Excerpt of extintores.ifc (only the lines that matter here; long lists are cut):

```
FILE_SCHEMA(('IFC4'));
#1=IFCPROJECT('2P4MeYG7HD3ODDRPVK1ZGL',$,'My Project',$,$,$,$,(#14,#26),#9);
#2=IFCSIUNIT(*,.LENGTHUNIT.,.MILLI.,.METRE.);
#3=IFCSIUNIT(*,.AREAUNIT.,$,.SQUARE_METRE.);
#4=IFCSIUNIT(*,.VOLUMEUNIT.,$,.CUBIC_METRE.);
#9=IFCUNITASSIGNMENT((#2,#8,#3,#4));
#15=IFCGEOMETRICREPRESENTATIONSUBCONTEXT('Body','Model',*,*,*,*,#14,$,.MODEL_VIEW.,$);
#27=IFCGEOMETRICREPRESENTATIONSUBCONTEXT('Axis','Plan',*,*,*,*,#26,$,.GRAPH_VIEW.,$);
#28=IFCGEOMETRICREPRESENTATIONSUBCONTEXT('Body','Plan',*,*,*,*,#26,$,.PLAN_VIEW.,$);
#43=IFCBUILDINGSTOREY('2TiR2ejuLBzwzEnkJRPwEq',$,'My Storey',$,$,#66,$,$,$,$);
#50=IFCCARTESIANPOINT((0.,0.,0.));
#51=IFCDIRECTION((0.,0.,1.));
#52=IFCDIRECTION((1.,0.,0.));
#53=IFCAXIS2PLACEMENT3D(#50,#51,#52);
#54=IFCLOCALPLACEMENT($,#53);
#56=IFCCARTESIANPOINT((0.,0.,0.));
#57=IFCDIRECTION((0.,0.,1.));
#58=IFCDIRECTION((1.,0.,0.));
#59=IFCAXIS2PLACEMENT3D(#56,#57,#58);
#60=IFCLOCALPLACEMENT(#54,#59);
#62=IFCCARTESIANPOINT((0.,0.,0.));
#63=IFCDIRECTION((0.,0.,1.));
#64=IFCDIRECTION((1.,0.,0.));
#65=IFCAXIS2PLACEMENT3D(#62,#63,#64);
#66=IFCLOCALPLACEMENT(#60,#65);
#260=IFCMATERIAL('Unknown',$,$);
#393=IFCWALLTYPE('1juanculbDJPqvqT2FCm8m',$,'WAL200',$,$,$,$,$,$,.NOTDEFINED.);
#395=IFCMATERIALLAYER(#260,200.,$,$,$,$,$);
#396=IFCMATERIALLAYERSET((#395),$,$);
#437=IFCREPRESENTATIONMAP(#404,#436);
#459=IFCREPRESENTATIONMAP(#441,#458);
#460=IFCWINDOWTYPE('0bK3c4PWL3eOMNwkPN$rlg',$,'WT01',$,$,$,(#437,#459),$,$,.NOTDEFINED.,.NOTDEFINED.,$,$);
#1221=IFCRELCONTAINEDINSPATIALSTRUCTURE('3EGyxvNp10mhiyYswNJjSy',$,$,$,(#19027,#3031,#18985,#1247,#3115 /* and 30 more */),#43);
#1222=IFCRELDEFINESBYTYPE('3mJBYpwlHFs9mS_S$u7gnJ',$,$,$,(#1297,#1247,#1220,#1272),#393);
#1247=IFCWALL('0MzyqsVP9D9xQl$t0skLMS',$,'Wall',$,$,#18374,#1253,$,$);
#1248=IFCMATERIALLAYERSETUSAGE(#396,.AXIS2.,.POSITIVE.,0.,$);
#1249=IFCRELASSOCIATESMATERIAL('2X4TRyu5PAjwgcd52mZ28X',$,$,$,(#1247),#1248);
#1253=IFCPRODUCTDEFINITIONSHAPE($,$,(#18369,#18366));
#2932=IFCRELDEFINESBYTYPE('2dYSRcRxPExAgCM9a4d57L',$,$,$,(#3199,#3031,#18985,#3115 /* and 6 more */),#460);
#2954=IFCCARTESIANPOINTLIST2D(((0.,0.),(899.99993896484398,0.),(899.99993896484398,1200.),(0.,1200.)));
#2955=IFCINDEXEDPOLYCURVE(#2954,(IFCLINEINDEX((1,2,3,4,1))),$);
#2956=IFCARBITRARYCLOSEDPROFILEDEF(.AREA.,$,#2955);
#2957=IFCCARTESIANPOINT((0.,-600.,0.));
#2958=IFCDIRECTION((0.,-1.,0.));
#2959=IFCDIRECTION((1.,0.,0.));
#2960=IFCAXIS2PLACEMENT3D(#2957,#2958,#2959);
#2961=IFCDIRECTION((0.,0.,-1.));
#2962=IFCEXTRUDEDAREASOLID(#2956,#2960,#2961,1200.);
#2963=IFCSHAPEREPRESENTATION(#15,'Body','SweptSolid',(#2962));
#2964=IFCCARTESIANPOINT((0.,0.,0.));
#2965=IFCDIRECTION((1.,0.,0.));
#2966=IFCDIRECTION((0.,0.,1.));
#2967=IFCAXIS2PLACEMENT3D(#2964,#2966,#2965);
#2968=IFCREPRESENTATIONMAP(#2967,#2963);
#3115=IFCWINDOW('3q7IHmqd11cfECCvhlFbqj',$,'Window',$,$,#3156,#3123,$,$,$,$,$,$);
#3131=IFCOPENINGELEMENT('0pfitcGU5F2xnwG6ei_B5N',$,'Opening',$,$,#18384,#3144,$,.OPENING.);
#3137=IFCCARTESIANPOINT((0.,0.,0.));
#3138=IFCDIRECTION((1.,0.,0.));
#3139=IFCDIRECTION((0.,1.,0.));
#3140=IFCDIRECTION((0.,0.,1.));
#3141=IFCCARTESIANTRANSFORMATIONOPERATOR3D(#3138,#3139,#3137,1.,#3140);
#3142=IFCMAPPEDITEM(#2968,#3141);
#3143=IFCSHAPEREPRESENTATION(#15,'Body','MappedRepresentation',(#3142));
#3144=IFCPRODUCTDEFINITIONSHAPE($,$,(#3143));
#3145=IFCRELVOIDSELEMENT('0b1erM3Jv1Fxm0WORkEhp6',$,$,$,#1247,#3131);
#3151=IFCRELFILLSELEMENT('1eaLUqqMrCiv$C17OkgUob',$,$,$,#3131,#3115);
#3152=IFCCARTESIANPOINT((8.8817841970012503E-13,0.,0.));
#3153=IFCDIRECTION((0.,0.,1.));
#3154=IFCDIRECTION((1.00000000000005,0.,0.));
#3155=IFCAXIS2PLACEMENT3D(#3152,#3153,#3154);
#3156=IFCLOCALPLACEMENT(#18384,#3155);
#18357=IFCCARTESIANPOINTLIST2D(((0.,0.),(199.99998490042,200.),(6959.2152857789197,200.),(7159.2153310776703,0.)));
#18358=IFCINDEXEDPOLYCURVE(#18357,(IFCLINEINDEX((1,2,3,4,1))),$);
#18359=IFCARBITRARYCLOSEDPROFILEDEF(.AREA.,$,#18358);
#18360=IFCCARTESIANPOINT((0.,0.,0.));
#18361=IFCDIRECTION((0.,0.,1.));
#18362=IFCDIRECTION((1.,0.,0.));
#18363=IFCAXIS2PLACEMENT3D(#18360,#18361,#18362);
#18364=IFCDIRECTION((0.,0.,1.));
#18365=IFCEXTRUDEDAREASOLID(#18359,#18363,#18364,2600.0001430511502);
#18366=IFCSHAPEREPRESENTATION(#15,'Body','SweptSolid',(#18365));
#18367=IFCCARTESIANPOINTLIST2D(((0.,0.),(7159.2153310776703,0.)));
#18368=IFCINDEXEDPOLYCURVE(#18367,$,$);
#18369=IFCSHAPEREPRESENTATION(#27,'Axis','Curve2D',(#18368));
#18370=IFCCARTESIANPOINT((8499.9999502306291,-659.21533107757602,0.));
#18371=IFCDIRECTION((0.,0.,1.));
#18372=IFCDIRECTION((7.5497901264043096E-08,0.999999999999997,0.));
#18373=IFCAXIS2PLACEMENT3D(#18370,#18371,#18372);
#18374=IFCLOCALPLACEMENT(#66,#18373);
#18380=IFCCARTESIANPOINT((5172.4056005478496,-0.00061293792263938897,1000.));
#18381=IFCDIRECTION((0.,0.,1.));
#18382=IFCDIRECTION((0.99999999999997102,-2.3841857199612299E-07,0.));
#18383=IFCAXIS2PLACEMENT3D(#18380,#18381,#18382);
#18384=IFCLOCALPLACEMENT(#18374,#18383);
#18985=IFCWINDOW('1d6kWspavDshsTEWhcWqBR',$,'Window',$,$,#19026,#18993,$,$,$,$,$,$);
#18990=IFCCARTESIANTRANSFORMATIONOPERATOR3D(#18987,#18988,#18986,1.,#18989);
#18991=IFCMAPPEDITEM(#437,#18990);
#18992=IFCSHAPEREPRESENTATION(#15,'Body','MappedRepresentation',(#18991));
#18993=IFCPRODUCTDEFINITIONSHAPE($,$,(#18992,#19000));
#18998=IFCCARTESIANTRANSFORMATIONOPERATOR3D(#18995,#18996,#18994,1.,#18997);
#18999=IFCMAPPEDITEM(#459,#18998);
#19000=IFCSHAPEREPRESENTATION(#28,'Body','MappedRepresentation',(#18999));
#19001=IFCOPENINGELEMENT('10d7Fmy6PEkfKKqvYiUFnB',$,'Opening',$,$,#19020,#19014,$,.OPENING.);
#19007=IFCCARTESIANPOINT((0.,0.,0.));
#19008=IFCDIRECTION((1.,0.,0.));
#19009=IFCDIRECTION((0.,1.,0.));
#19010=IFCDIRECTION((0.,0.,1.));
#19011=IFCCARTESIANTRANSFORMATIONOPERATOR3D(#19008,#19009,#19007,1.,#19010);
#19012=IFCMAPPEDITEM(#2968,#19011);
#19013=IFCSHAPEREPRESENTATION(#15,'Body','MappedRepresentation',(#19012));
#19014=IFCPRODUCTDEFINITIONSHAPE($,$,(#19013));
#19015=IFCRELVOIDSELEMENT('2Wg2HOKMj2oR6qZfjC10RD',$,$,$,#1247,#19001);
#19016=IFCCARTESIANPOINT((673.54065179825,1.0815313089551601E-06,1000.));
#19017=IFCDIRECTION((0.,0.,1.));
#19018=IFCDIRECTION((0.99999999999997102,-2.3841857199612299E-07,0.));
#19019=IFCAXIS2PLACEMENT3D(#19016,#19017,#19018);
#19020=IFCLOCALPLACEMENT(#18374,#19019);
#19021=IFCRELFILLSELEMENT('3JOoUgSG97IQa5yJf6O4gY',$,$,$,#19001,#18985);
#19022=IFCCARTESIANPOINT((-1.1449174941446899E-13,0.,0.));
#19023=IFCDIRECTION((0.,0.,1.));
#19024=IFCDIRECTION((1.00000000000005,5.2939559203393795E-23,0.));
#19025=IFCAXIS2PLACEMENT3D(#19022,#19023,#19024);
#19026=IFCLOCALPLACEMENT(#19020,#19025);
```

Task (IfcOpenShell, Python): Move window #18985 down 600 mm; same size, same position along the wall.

```python
import numpy as np
import ifcopenshell
import ifcopenshell.api.geometry
import ifcopenshell.util.placement
import ifcopenshell.util.unit

model = ifcopenshell.open("extintores.ifc")
unit_scale = ifcopenshell.util.unit.calculate_unit_scale(model)

window = model.by_guid("1d6kWspavDshsTEWhcWqBR")
opening = window.FillsVoids[0].RelatingOpeningElement
dz = -0.6 / unit_scale

shift = np.array([0.0, 0.0, dz])
# The window is placed relative to its opening, so it follows when the opening moves.
matrix = ifcopenshell.util.placement.get_local_placement(opening.ObjectPlacement)
matrix[:3, 3] += shift
ifcopenshell.api.geometry.edit_object_placement(
    model, product=opening, matrix=matrix, is_si=False, should_transform_children=True
)

print(f"moved by {dz * unit_scale:+.3f} m")

model.write("extintores-out.ifc")
```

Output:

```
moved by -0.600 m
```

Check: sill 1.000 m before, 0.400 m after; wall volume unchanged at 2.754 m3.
